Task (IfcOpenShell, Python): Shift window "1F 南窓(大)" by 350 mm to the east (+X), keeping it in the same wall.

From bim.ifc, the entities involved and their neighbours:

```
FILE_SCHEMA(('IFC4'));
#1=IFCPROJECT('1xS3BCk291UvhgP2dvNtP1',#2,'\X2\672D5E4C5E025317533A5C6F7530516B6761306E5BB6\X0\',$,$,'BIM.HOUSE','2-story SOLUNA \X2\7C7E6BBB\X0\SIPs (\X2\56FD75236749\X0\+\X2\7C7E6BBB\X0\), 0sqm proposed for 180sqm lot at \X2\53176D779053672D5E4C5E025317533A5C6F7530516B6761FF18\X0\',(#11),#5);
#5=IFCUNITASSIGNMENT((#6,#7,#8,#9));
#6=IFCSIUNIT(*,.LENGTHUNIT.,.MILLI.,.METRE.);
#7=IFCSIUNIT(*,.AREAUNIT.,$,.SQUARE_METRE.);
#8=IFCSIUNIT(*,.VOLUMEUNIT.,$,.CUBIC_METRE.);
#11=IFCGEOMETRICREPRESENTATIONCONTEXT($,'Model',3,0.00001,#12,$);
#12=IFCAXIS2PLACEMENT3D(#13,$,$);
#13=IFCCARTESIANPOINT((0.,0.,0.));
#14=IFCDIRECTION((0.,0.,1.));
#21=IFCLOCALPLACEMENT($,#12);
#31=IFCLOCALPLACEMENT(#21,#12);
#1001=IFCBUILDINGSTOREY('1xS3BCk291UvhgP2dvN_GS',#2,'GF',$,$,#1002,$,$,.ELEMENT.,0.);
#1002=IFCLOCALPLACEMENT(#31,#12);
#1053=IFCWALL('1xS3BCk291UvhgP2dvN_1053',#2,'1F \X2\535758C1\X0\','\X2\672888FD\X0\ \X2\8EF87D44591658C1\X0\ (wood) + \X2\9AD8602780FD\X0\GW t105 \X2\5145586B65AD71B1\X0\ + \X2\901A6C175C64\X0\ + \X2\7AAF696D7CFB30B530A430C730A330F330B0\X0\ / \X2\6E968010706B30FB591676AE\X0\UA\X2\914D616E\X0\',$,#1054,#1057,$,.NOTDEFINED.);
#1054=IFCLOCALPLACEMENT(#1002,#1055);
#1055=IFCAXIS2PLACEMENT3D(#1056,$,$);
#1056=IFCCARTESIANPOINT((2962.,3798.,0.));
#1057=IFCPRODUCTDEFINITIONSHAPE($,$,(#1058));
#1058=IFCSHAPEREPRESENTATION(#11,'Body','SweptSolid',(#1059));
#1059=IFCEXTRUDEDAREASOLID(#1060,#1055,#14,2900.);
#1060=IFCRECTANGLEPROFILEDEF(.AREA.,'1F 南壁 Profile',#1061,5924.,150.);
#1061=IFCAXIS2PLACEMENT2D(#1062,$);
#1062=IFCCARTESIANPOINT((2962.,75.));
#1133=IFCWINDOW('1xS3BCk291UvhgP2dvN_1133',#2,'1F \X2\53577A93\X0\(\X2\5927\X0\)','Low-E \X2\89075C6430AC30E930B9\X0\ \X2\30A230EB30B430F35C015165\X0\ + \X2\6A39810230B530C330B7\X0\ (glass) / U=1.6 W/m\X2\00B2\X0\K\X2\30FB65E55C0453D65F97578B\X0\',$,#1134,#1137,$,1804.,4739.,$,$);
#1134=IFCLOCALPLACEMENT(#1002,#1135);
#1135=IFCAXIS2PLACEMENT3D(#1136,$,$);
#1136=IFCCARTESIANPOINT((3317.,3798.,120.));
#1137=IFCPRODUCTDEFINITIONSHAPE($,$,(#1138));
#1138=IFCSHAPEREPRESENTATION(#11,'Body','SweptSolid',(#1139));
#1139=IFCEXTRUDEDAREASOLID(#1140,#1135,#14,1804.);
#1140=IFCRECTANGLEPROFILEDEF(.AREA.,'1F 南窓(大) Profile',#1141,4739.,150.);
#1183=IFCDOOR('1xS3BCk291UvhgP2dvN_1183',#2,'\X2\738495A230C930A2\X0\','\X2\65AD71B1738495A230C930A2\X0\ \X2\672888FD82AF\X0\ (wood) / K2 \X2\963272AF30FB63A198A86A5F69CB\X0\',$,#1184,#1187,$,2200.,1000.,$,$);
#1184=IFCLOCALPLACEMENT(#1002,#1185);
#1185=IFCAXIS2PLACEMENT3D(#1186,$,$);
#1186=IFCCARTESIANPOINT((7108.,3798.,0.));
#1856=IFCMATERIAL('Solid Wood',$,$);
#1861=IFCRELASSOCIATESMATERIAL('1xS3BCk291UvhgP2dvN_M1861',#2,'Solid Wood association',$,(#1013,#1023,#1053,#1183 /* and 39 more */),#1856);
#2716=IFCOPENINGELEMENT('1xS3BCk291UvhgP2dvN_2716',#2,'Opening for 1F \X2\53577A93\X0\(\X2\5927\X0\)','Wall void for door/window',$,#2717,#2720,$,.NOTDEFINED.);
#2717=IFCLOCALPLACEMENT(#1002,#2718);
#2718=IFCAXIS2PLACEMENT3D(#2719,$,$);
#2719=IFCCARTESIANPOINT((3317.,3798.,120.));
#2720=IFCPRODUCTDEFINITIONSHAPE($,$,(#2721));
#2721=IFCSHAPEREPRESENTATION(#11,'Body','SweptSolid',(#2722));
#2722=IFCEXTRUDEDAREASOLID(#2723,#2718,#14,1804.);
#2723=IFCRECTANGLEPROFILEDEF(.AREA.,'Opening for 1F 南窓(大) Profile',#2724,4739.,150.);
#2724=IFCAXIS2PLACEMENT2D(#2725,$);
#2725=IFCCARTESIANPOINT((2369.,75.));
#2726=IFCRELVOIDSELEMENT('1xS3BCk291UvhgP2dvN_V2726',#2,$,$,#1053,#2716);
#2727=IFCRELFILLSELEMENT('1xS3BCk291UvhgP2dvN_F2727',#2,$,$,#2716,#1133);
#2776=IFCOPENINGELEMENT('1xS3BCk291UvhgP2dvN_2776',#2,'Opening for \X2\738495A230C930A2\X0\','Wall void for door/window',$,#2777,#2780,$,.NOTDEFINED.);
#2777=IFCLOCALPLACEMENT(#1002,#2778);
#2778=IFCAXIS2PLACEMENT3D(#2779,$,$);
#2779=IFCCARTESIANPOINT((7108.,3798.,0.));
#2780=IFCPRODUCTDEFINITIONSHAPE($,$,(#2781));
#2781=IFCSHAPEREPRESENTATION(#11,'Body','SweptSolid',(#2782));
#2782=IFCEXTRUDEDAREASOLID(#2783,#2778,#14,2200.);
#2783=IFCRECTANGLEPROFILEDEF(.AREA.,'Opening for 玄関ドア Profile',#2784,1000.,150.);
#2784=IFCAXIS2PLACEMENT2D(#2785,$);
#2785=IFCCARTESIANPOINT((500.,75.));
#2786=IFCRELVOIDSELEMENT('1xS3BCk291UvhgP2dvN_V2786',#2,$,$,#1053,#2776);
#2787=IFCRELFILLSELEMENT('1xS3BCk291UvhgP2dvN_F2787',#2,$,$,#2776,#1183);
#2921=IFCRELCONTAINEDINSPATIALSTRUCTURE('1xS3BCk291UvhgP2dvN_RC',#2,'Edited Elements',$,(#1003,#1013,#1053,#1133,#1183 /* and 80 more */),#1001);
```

```python
import ifcopenshell
import ifcopenshell.api.geometry
import ifcopenshell.util.placement
import ifcopenshell.util.unit

model = ifcopenshell.open("bim.ifc")
unit_scale = ifcopenshell.util.unit.calculate_unit_scale(model)

window = model.by_guid("1xS3BCk291UvhgP2dvN_1133")
opening = window.FillsVoids[0].RelatingOpeningElement
wall = opening.VoidsElements[0].RelatingBuildingElement

wall_matrix = ifcopenshell.util.placement.get_local_placement(wall.ObjectPlacement)
shift = wall_matrix[:3, 0] * 0.35 / unit_scale
before = ifcopenshell.util.placement.get_local_placement(window.ObjectPlacement)[:3, 3].copy()

# The window is not placed relative to its opening, so move both.
for product in (opening, window):
    matrix = ifcopenshell.util.placement.get_local_placement(product.ObjectPlacement)
    matrix[:3, 3] += shift
    ifcopenshell.api.geometry.edit_object_placement(model, product=product, matrix=matrix, is_si=False)

after = ifcopenshell.util.placement.get_local_placement(window.ObjectPlacement)[:3, 3]
print("window moved by", (after - before).round(3) + 0.0)

model.write("bim_v2.ifc")
```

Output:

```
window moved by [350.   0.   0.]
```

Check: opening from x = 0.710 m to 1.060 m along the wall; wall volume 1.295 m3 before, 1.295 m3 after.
